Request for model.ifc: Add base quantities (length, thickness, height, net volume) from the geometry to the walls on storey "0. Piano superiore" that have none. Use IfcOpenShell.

First a look at what the model holds.

```python
import ifcopenshell
import ifcopenshell.util.element
import ifcopenshell.util.unit

model = ifcopenshell.open("model.ifc")
print(model.schema)
for unit_type in ("LENGTHUNIT", "AREAUNIT", "VOLUMEUNIT"):
    print(unit_type, ifcopenshell.util.unit.calculate_unit_scale(model, unit_type))
storey = next(s for s in model.by_type("IfcBuildingStorey") if s.Name == "0. Piano superiore")
walls = [e for e in ifcopenshell.util.element.get_decomposition(storey) if e.is_a("IfcWall")]
for e in sorted(walls, key=lambda e: e.id()):
    print(e.id(), e.is_a(), e.Name, list(ifcopenshell.util.element.get_psets(e, qtos_only=True)), sep=" | ")
```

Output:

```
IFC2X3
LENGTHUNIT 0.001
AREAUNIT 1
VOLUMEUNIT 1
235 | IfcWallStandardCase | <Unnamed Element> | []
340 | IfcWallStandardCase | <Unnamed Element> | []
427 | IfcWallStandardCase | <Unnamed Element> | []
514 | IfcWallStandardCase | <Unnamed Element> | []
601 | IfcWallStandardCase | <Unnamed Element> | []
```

```python
import ifcopenshell
import ifcopenshell.api.pset
import ifcopenshell.geom
import ifcopenshell.util.element
import ifcopenshell.util.shape
import ifcopenshell.util.unit

model = ifcopenshell.open("model.ifc")
unit_scale = ifcopenshell.util.unit.calculate_unit_scale(model)
volume_scale = ifcopenshell.util.unit.calculate_unit_scale(model, "VOLUMEUNIT")
settings = ifcopenshell.geom.settings()

storey = next(s for s in model.by_type("IfcBuildingStorey") if s.Name == "0. Piano superiore")
walls = [e for e in ifcopenshell.util.element.get_decomposition(storey) if e.is_a("IfcWall")]

for e in sorted(walls, key=lambda e: e.id()):
    if ifcopenshell.util.element.get_psets(e, qtos_only=True, should_inherit=False):
        continue
    # Geometry comes back in metres, in the element's own axes.
    shape = ifcopenshell.geom.create_shape(settings, e)
    values = {
        "Length": ifcopenshell.util.shape.get_x(shape.geometry) / unit_scale,
        "Width": ifcopenshell.util.shape.get_y(shape.geometry) / unit_scale,
        "Height": ifcopenshell.util.shape.get_z(shape.geometry) / unit_scale,
        "NetVolume": ifcopenshell.util.shape.get_volume(shape.geometry) / volume_scale,
    }
    qto = ifcopenshell.api.pset.add_qto(model, product=e, name="BaseQuantities")
    ifcopenshell.api.pset.edit_qto(model, qto=qto, properties=values)
    print(e.id(), {k: round(v, 3) for k, v in values.items()})

model.write("model_edited.ifc")
```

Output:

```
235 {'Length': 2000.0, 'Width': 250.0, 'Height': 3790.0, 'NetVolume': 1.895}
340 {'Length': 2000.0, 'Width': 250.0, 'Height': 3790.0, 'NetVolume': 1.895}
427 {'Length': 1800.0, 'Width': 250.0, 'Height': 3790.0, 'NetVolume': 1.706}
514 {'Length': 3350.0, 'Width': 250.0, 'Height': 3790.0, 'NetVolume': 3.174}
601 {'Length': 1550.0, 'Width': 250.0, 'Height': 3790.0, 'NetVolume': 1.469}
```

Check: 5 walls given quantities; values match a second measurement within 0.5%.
